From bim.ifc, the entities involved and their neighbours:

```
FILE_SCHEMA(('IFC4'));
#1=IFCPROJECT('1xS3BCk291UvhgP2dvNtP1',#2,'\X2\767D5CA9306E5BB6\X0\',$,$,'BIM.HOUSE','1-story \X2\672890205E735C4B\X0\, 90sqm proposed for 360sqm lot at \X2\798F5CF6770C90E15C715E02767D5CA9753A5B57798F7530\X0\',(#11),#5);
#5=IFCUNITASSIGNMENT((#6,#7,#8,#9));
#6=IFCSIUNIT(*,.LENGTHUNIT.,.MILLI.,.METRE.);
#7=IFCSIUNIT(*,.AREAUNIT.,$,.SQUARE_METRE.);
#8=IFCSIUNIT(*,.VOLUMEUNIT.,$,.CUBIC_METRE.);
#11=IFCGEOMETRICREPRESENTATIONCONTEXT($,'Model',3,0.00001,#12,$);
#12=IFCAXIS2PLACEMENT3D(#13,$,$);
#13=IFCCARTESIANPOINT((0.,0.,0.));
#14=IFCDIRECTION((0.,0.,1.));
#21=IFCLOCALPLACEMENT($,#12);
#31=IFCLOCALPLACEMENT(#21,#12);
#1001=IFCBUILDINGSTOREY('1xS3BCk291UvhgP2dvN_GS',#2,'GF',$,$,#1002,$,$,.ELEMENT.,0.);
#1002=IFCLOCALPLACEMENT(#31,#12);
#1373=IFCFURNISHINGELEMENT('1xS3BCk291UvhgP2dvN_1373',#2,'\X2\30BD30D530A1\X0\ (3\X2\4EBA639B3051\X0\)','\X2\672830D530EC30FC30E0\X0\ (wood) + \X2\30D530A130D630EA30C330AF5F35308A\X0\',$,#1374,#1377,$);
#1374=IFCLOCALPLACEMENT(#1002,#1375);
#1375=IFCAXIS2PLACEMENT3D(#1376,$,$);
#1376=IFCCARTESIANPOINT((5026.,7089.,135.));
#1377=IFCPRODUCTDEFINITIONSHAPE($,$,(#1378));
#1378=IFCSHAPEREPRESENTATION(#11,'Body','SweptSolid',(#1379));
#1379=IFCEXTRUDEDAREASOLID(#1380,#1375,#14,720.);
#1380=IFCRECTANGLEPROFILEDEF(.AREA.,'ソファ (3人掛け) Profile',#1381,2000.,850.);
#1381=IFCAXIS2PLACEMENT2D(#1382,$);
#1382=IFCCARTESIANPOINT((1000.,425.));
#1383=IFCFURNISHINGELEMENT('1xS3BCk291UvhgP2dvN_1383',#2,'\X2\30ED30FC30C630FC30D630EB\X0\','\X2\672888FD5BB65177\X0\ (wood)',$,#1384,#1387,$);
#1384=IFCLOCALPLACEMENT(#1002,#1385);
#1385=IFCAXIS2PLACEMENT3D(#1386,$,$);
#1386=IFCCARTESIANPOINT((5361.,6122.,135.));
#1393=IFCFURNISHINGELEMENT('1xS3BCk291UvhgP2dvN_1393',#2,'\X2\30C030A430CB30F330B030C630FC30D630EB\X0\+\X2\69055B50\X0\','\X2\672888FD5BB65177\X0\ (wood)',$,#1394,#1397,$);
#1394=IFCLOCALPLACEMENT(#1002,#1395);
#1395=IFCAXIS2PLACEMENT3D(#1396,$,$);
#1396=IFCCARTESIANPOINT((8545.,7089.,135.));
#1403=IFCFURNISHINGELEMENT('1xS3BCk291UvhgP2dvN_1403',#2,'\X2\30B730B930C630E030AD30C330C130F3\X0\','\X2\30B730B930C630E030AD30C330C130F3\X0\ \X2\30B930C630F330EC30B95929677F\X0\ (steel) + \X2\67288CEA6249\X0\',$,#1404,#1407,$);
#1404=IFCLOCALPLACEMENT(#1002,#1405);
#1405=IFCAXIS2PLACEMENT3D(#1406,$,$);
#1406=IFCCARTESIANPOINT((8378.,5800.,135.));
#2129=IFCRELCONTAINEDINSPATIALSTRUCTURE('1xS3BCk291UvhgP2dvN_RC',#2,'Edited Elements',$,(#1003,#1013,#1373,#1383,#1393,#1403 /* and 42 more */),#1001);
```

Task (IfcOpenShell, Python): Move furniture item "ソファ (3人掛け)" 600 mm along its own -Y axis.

```python
import ifcopenshell
import ifcopenshell.api.geometry
import ifcopenshell.util.placement

model = ifcopenshell.open("bim.ifc")

item = model.by_guid("1xS3BCk291UvhgP2dvN_1373")
matrix = ifcopenshell.util.placement.get_local_placement(item.ObjectPlacement)
matrix[:3, 3] -= matrix[:3, 1] * 600.0
ifcopenshell.api.geometry.edit_object_placement(model, product=item, matrix=matrix, is_si=False)

print(ifcopenshell.util.placement.get_local_placement(item.ObjectPlacement).round(3) + 0.0)

model.write("bim_updated.ifc")
```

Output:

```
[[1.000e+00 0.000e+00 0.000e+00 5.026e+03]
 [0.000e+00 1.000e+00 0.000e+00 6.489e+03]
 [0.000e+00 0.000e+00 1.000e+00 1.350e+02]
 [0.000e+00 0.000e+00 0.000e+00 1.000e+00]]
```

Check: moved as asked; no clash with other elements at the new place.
